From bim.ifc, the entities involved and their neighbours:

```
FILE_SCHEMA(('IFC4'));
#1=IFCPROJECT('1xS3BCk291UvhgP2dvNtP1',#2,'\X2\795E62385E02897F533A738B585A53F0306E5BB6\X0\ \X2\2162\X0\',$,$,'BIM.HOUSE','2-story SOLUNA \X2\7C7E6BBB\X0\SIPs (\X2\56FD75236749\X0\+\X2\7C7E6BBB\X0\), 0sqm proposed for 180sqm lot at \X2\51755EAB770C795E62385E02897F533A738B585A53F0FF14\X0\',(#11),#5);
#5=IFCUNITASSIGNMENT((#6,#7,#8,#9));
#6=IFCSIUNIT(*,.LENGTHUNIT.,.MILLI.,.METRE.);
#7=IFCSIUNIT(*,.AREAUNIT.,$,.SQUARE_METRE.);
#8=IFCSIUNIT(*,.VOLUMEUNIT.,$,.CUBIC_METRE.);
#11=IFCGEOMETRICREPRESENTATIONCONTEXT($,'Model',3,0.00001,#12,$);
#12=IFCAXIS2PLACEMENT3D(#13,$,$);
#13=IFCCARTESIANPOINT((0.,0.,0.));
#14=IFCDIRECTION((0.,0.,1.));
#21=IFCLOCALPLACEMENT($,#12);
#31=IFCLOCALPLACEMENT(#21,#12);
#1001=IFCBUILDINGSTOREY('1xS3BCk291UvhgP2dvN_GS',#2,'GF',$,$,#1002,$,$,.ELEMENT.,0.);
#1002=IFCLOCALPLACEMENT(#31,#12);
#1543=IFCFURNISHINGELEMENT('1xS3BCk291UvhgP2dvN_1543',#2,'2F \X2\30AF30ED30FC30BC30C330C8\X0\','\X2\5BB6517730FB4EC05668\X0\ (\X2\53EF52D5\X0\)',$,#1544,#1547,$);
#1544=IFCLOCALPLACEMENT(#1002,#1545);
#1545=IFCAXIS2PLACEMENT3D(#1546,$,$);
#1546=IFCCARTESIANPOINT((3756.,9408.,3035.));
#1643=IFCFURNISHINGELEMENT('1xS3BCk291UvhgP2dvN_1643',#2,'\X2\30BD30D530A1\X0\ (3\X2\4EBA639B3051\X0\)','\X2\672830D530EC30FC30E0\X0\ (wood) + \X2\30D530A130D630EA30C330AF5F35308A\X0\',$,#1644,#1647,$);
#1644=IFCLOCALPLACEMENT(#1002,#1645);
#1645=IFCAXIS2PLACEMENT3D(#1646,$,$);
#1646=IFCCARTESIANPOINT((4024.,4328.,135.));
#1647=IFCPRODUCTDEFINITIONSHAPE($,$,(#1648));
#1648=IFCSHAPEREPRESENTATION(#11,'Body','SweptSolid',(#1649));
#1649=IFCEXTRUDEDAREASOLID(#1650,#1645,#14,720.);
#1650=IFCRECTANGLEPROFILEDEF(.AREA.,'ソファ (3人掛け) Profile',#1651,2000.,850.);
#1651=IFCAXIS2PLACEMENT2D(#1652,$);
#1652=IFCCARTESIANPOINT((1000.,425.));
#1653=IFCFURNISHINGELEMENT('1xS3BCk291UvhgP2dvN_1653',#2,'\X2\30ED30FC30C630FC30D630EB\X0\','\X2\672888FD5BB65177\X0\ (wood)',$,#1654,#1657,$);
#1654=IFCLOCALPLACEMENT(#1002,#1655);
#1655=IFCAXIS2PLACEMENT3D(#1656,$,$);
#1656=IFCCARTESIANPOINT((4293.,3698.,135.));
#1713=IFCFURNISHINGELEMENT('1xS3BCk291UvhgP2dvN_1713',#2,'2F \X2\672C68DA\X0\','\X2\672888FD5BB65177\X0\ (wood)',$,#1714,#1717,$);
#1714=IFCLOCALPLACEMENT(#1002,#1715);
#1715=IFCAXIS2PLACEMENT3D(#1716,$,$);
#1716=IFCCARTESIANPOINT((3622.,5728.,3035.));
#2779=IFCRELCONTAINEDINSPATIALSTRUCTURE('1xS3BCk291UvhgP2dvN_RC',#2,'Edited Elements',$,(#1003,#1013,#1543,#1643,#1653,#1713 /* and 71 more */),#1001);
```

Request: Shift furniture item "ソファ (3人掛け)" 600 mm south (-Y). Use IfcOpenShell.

```python
import ifcopenshell
import ifcopenshell.api.geometry
import ifcopenshell.util.placement
import ifcopenshell.util.unit

model = ifcopenshell.open("bim.ifc")
unit_scale = ifcopenshell.util.unit.calculate_unit_scale(model)

item = model.by_guid("1xS3BCk291UvhgP2dvN_1643")
matrix = ifcopenshell.util.placement.get_local_placement(item.ObjectPlacement)
matrix[1, 3] -= 0.6 / unit_scale
ifcopenshell.api.geometry.edit_object_placement(model, product=item, matrix=matrix, is_si=False)

print(ifcopenshell.util.placement.get_local_placement(item.ObjectPlacement).round(3) + 0.0)

model.write("bim_edited.ifc")
```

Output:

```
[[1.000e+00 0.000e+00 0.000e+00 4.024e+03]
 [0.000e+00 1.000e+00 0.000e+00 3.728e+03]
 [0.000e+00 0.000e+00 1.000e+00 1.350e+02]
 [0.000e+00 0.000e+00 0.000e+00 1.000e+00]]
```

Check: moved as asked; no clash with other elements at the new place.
